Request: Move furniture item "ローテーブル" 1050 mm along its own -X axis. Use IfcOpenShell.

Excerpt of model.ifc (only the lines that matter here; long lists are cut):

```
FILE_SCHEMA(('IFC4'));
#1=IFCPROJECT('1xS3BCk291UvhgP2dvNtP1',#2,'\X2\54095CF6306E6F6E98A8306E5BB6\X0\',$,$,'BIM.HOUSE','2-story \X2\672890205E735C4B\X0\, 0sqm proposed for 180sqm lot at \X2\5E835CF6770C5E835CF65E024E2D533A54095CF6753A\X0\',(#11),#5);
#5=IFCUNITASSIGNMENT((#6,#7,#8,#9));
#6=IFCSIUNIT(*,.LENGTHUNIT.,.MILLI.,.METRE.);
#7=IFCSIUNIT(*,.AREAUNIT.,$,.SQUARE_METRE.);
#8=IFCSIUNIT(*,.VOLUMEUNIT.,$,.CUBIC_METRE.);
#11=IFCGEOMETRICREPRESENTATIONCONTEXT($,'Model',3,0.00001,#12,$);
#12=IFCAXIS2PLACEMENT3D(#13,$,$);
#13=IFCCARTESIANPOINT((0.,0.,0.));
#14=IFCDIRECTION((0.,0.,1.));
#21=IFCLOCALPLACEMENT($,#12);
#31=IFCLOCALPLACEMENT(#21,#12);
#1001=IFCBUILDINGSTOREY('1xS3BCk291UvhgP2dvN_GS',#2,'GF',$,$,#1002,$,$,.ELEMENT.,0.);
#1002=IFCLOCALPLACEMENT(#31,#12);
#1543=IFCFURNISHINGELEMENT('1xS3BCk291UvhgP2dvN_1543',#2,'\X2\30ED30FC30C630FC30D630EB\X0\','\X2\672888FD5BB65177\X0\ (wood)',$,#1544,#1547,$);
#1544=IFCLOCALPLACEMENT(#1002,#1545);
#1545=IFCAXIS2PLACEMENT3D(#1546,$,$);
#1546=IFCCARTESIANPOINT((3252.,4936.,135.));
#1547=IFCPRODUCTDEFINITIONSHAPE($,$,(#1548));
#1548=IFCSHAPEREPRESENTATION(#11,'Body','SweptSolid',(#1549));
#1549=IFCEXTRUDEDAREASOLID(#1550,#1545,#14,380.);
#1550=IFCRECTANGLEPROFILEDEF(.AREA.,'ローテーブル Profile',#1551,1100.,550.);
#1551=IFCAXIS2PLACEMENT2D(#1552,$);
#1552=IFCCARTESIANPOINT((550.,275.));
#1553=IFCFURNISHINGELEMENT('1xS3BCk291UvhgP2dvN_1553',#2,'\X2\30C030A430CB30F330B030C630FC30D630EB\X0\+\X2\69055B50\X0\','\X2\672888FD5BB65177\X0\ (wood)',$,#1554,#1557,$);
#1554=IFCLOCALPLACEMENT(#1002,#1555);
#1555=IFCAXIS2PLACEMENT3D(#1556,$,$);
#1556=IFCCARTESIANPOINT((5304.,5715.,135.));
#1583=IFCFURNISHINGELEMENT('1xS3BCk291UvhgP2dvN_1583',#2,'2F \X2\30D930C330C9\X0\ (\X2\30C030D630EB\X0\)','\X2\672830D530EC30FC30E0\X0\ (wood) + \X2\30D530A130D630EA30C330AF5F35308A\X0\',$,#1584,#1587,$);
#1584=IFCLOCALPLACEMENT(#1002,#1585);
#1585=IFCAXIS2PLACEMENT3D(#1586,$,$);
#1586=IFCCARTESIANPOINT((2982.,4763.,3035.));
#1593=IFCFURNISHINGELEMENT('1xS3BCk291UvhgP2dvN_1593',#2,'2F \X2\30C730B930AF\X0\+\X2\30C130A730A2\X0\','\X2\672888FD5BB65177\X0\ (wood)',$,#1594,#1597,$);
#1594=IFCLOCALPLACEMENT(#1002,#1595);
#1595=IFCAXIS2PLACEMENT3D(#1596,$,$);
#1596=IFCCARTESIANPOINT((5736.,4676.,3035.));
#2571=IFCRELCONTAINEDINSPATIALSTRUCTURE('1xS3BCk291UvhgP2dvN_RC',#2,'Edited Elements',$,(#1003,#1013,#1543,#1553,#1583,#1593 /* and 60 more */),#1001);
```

```python
import ifcopenshell
import ifcopenshell.api.geometry
import ifcopenshell.util.placement

model = ifcopenshell.open("model.ifc")

item = model.by_guid("1xS3BCk291UvhgP2dvN_1543")
matrix = ifcopenshell.util.placement.get_local_placement(item.ObjectPlacement)
matrix[:3, 3] -= matrix[:3, 0] * 1050.0
ifcopenshell.api.geometry.edit_object_placement(model, product=item, matrix=matrix, is_si=False)

print(ifcopenshell.util.placement.get_local_placement(item.ObjectPlacement).round(3) + 0.0)

model.write("model_rev.ifc")
```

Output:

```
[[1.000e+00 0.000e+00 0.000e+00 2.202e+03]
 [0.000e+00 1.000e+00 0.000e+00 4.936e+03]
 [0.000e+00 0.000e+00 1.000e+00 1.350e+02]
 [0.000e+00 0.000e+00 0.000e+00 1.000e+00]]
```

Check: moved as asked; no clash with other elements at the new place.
